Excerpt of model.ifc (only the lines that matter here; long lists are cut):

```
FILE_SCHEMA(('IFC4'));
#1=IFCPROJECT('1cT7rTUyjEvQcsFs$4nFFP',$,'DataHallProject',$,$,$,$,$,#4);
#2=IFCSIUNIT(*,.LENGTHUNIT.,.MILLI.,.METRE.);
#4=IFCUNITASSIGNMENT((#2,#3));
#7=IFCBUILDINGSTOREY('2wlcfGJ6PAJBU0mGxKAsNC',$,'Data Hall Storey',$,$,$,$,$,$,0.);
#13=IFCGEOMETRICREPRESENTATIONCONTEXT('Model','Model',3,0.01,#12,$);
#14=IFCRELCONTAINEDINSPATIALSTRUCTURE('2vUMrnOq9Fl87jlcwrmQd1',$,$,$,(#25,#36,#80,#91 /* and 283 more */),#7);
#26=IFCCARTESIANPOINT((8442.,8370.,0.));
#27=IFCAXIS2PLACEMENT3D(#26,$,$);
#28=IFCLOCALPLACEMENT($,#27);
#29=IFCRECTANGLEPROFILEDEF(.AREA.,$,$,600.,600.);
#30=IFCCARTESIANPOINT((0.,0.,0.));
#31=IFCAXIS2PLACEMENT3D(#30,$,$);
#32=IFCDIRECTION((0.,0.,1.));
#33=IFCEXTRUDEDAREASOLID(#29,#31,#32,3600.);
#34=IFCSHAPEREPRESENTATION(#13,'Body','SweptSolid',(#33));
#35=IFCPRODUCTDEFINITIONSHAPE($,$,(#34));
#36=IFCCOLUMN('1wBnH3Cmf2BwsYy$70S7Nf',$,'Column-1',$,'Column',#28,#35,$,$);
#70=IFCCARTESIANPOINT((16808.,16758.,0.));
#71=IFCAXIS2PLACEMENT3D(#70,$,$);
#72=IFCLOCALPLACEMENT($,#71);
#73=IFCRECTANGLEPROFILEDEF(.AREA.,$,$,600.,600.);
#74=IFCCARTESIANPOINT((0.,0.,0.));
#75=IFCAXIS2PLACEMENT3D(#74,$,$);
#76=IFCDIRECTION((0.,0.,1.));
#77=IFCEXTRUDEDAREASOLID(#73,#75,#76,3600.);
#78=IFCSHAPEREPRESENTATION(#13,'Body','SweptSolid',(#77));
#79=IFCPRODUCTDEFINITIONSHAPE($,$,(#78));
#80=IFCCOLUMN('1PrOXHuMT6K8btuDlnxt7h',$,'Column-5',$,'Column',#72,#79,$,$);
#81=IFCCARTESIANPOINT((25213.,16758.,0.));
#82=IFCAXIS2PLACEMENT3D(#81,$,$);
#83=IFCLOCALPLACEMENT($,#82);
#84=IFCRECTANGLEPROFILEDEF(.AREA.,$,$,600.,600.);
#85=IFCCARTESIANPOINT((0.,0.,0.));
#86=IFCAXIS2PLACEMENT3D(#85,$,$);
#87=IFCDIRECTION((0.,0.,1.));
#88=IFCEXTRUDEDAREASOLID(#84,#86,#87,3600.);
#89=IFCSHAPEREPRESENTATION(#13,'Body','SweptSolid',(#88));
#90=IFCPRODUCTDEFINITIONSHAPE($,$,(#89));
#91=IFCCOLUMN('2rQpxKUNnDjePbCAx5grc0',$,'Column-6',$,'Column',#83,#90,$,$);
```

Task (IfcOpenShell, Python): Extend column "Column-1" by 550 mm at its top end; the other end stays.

```python
import ifcopenshell

model = ifcopenshell.open("model.ifc")

member = model.by_guid("1wBnH3Cmf2BwsYy$70S7Nf")
change = 550.0

# The extrusion runs towards the end named, so only its depth changes.
body = next(r for r in member.Representation.Representations if r.RepresentationIdentifier == "Body")
solid = body.Items[0]
old_length = solid.Depth
solid.Depth += change

print(f"length {old_length:g} -> {solid.Depth:g}")

model.write("model-out.ifc")
```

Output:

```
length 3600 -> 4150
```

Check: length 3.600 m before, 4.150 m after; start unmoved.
